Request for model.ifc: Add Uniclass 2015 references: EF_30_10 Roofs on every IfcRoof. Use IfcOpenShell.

First a look at what the model holds.

```python
import ifcopenshell

model = ifcopenshell.open("model.ifc")
print(model.schema)
print("classifications:", [c.Name for c in model.by_type("IfcClassification")])
for ifc_class in ("IfcDoor", "IfcRoof", "IfcStair", "IfcWall", "IfcWindow"):
    print(ifc_class, len(model.by_type(ifc_class)))
```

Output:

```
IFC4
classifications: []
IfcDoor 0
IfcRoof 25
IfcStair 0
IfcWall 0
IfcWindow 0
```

```python
import ifcopenshell
import ifcopenshell.api.classification

model = ifcopenshell.open("model.ifc")

system = ifcopenshell.api.classification.add_classification(model, classification="Uniclass 2015")

codes = {
    "IfcRoof": ("EF_30_10", "Roofs"),
}
for ifc_class, (code, name) in codes.items():
    products = model.by_type(ifc_class)
    ifcopenshell.api.classification.add_reference(
        model, products=products, classification=system, identification=code, name=name
    )
    print(code, len(products))

model.write("model_v2.ifc")
```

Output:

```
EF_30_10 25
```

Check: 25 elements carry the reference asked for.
